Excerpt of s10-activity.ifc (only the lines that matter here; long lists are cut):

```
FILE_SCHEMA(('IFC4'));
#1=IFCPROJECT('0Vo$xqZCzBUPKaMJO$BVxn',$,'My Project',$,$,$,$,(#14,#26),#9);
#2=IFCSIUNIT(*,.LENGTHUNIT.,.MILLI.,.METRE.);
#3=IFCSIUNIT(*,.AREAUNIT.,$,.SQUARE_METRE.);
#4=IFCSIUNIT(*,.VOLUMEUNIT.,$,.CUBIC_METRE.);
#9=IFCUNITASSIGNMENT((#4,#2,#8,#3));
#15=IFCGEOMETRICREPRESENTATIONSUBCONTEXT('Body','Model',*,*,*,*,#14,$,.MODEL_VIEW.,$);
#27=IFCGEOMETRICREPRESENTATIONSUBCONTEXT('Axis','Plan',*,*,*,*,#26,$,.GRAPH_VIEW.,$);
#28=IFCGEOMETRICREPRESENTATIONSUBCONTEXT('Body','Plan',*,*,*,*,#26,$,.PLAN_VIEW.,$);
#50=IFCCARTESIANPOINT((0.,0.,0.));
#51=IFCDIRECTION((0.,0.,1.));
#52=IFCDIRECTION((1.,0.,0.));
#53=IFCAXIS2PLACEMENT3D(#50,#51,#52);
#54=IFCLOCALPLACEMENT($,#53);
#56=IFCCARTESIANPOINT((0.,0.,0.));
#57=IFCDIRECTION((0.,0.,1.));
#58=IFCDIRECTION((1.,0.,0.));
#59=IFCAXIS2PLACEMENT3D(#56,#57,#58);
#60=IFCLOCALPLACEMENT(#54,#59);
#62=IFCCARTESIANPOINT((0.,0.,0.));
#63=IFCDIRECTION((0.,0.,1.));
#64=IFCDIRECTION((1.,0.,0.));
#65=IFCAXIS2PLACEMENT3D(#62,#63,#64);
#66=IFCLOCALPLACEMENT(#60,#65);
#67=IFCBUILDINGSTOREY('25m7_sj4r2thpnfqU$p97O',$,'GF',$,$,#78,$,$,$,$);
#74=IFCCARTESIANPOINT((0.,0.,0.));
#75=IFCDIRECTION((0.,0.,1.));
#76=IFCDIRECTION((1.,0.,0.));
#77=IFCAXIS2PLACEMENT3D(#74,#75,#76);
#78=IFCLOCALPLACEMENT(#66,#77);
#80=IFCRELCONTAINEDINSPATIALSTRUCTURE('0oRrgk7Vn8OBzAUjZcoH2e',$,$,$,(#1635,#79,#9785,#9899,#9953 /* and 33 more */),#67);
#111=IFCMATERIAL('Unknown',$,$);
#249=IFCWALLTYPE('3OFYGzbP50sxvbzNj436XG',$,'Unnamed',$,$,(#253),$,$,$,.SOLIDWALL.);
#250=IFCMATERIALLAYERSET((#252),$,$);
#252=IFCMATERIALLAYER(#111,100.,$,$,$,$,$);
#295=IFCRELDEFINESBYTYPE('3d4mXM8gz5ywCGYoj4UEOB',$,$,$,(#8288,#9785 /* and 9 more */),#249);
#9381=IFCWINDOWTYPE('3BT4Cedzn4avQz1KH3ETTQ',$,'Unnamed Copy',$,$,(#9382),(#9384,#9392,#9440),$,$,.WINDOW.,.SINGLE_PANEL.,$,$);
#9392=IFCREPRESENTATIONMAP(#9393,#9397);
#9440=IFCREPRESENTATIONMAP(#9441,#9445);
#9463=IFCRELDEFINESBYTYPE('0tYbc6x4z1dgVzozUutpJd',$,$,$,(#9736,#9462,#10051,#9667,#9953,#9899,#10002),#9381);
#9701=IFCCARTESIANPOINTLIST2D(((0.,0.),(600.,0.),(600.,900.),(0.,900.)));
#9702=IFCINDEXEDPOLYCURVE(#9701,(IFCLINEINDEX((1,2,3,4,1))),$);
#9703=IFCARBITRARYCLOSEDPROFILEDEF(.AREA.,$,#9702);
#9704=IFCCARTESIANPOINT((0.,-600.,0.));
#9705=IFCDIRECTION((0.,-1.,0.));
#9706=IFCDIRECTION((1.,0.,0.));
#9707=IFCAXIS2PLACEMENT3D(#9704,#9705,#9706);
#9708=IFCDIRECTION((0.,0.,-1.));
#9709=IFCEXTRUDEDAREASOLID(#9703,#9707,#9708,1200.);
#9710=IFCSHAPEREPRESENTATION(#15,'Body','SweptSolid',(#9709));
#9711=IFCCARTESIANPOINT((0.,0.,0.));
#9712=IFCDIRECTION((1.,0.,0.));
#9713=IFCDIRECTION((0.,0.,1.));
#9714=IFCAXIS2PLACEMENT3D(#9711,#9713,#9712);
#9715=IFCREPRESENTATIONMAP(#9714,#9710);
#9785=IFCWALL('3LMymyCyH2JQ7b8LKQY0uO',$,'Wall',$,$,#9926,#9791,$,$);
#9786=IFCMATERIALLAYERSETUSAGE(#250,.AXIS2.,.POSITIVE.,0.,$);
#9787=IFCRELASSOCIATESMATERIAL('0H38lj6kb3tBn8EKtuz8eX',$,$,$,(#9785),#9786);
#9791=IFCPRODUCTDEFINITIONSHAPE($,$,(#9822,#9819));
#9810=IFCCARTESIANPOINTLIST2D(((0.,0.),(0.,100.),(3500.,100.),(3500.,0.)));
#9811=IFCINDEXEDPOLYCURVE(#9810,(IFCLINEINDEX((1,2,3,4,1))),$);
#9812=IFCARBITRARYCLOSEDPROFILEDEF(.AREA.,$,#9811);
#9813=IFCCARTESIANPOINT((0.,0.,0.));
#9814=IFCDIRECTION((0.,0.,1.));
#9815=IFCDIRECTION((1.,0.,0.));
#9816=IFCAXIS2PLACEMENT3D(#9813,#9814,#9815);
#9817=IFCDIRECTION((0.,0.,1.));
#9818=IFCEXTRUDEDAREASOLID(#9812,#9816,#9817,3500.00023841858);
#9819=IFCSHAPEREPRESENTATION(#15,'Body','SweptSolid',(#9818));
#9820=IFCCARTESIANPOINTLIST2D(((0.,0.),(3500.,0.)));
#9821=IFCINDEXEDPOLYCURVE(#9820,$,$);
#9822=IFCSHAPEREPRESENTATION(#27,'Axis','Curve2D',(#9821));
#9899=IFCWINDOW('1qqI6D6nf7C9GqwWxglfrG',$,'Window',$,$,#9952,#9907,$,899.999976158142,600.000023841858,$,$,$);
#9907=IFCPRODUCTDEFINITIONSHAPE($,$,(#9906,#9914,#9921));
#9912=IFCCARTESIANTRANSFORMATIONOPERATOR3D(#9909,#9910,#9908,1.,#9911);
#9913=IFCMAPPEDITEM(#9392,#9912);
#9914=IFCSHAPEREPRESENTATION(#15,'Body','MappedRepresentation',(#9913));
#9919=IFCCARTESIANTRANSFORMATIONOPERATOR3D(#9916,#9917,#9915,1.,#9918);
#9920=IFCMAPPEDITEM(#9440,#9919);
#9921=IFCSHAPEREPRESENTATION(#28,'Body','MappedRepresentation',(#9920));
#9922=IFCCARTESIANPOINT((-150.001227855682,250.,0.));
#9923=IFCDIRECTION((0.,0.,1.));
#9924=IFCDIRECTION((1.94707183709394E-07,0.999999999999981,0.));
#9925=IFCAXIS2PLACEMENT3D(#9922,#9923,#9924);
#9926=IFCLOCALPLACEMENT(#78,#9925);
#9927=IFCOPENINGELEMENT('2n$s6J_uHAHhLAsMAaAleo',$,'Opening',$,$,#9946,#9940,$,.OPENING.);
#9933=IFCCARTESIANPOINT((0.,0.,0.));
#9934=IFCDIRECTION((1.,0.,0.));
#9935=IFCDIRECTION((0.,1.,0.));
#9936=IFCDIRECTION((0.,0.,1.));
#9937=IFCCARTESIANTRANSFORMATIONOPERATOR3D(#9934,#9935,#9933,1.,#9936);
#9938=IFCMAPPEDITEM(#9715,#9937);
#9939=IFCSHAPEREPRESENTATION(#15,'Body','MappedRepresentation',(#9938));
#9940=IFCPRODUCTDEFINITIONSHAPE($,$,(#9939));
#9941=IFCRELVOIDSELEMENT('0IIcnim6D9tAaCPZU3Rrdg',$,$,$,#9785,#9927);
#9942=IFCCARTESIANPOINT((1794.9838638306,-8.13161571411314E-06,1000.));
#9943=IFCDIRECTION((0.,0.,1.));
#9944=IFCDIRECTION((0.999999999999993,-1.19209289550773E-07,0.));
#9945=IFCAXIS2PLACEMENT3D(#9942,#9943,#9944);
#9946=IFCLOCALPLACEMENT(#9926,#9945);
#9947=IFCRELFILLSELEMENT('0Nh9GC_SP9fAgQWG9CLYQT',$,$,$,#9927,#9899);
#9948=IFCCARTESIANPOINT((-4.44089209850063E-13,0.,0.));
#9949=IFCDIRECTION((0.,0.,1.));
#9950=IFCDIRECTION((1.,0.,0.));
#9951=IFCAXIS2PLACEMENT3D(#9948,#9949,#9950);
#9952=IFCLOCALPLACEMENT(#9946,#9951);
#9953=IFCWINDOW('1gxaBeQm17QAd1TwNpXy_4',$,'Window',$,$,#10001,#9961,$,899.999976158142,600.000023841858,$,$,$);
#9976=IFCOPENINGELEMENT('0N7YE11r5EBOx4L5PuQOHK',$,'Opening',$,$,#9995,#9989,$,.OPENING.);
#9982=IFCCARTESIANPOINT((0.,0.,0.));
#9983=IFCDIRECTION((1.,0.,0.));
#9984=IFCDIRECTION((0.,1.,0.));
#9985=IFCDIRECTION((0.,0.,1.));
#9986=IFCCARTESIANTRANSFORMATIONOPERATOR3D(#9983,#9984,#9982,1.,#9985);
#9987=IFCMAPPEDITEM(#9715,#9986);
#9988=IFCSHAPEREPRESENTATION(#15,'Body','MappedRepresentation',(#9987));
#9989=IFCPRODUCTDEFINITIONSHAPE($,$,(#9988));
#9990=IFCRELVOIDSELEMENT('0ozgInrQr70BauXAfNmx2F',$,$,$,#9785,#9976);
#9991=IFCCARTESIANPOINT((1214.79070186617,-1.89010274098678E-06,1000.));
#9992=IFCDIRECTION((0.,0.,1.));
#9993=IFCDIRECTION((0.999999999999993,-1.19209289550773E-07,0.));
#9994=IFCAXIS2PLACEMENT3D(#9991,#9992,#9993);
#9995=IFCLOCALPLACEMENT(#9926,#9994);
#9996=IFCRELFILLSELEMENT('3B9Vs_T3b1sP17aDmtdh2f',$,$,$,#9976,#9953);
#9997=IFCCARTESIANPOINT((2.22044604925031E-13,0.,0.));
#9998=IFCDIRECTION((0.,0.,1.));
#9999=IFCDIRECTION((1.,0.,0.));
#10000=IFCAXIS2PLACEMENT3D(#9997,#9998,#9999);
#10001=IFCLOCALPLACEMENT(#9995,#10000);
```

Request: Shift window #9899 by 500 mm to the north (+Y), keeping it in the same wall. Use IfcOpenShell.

```python
import ifcopenshell
import ifcopenshell.api.geometry
import ifcopenshell.util.placement
import ifcopenshell.util.unit

model = ifcopenshell.open("s10-activity.ifc")
unit_scale = ifcopenshell.util.unit.calculate_unit_scale(model)

window = model.by_guid("1qqI6D6nf7C9GqwWxglfrG")
opening = window.FillsVoids[0].RelatingOpeningElement
wall = opening.VoidsElements[0].RelatingBuildingElement

wall_matrix = ifcopenshell.util.placement.get_local_placement(wall.ObjectPlacement)
shift = wall_matrix[:3, 0] * 0.5 / unit_scale
before = ifcopenshell.util.placement.get_local_placement(window.ObjectPlacement)[:3, 3].copy()

# The window is placed relative to its opening, so it follows when the opening moves.
matrix = ifcopenshell.util.placement.get_local_placement(opening.ObjectPlacement)
matrix[:3, 3] += shift
ifcopenshell.api.geometry.edit_object_placement(
    model, product=opening, matrix=matrix, is_si=False, should_transform_children=True
)

after = ifcopenshell.util.placement.get_local_placement(window.ObjectPlacement)[:3, 3]
print("window moved by", (after - before).round(3) + 0.0)

model.write("s10-activity_edited.ifc")
```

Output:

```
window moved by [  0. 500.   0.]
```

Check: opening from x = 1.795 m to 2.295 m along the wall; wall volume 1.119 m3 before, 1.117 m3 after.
